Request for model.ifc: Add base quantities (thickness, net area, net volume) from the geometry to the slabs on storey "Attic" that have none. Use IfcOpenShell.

First a look at what the model holds.

```python
import ifcopenshell
import ifcopenshell.util.element
import ifcopenshell.util.unit

model = ifcopenshell.open("model.ifc")
print(model.schema)
for unit_type in ("LENGTHUNIT", "AREAUNIT", "VOLUMEUNIT"):
    print(unit_type, ifcopenshell.util.unit.calculate_unit_scale(model, unit_type))
storey = next(s for s in model.by_type("IfcBuildingStorey") if s.Name == "Attic")
slabs = [e for e in ifcopenshell.util.element.get_decomposition(storey) if e.is_a("IfcSlab")]
for e in sorted(slabs, key=lambda e: e.id()):
    print(e.id(), e.is_a(), e.Name, list(ifcopenshell.util.element.get_psets(e, qtos_only=True)), sep=" | ")
```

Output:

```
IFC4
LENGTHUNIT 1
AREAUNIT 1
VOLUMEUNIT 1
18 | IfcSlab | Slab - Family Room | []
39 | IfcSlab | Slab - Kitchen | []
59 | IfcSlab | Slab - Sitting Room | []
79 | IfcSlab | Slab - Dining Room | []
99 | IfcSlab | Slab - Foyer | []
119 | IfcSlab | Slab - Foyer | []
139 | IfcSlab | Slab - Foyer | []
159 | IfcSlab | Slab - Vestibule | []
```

```python
import ifcopenshell
import ifcopenshell.api.pset
import ifcopenshell.geom
import ifcopenshell.util.element
import ifcopenshell.util.shape
import ifcopenshell.util.unit

model = ifcopenshell.open("model.ifc")
unit_scale = ifcopenshell.util.unit.calculate_unit_scale(model)
area_scale = ifcopenshell.util.unit.calculate_unit_scale(model, "AREAUNIT")
volume_scale = ifcopenshell.util.unit.calculate_unit_scale(model, "VOLUMEUNIT")
settings = ifcopenshell.geom.settings()

storey = next(s for s in model.by_type("IfcBuildingStorey") if s.Name == "Attic")
slabs = [e for e in ifcopenshell.util.element.get_decomposition(storey) if e.is_a("IfcSlab")]

for e in sorted(slabs, key=lambda e: e.id()):
    if ifcopenshell.util.element.get_psets(e, qtos_only=True, should_inherit=False):
        continue
    # Geometry comes back in metres, in the element's own axes.
    shape = ifcopenshell.geom.create_shape(settings, e)
    values = {
        "Width": ifcopenshell.util.shape.get_z(shape.geometry) / unit_scale,
        "NetArea": ifcopenshell.util.shape.get_footprint_area(shape.geometry) / area_scale,
        "NetVolume": ifcopenshell.util.shape.get_volume(shape.geometry) / volume_scale,
    }
    qto = ifcopenshell.api.pset.add_qto(model, product=e, name="Qto_SlabBaseQuantities")
    ifcopenshell.api.pset.edit_qto(model, qto=qto, properties=values)
    print(e.id(), {k: round(v, 3) for k, v in values.items()})

model.write("model_rev.ifc")
```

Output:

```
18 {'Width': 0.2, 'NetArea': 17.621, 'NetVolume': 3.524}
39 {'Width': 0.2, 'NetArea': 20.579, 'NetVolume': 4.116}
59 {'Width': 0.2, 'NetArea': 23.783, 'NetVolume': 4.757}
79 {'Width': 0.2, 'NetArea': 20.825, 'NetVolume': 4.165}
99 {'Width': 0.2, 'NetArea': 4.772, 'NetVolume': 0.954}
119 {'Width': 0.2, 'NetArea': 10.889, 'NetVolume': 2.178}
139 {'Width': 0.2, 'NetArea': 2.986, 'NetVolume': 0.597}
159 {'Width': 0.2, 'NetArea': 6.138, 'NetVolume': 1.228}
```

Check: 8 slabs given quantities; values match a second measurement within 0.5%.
